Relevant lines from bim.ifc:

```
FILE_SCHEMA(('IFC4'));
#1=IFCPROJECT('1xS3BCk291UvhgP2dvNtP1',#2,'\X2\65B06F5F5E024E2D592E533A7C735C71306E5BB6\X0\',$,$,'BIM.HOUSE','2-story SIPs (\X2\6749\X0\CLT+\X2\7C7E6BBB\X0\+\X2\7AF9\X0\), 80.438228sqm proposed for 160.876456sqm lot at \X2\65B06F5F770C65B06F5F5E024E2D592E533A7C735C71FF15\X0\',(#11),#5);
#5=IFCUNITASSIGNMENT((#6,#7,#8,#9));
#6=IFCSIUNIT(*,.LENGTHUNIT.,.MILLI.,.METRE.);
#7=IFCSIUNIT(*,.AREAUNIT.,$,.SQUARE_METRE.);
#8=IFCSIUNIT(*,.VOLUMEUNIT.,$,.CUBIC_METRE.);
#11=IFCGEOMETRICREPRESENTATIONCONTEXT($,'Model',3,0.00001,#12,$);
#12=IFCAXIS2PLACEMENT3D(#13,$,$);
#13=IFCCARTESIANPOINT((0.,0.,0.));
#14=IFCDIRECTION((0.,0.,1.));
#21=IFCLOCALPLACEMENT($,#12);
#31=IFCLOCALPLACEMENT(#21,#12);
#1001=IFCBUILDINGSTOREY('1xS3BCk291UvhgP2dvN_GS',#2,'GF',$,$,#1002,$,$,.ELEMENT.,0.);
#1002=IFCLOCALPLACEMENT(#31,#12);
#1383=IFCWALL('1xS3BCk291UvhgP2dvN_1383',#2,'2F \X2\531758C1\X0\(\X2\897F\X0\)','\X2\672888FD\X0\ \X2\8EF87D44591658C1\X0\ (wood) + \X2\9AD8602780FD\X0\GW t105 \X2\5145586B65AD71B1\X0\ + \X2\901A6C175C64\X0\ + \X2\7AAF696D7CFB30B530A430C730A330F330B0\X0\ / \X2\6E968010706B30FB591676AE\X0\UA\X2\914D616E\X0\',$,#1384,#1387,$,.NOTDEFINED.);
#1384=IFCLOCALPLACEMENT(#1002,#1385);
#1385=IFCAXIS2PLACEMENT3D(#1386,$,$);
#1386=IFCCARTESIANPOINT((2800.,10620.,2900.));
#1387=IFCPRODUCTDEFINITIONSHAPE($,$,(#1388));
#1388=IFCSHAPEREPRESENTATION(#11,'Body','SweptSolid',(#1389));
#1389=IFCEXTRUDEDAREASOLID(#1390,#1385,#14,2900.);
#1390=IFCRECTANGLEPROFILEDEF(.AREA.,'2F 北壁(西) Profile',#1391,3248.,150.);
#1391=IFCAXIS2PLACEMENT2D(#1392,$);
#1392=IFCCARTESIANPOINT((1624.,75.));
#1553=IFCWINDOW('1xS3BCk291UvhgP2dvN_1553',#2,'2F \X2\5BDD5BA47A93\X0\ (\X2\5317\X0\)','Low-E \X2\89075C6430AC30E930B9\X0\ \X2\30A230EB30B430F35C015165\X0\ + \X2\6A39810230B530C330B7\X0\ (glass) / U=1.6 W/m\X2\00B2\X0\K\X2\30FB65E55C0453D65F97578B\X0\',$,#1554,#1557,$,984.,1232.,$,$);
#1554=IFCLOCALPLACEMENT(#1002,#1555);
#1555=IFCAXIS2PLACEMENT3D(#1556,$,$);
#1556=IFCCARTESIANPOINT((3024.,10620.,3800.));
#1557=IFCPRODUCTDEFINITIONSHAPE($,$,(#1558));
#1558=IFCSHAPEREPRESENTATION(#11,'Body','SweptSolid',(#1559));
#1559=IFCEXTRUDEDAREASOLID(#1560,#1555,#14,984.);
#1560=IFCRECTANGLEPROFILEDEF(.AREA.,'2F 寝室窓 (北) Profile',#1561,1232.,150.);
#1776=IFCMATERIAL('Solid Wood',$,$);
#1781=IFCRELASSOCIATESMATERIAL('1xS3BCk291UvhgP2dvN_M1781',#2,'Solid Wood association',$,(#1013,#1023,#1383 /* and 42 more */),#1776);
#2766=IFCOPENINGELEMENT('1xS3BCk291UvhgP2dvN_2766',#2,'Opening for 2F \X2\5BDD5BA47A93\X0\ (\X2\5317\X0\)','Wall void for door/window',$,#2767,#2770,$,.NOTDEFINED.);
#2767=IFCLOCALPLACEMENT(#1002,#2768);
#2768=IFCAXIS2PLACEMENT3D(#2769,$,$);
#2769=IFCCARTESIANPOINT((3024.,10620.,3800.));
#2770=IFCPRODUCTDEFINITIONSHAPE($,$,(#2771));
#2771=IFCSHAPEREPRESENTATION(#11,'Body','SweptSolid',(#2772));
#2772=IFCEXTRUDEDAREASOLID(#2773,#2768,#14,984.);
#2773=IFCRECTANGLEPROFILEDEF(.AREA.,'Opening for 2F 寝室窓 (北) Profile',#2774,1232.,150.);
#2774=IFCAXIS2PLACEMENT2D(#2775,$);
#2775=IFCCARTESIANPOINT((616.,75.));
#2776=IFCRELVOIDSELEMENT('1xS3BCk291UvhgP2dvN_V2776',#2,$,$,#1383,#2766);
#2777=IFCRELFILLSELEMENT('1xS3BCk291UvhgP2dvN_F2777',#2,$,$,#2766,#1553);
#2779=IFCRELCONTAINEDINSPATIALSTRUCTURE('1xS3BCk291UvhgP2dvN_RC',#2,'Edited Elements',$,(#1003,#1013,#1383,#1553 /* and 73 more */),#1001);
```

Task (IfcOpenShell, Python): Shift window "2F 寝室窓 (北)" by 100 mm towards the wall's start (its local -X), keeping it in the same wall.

```python
import ifcopenshell
import ifcopenshell.api.geometry
import ifcopenshell.util.placement
import ifcopenshell.util.unit

model = ifcopenshell.open("bim.ifc")
unit_scale = ifcopenshell.util.unit.calculate_unit_scale(model)

window = model.by_guid("1xS3BCk291UvhgP2dvN_1553")
opening = window.FillsVoids[0].RelatingOpeningElement
wall = opening.VoidsElements[0].RelatingBuildingElement

wall_matrix = ifcopenshell.util.placement.get_local_placement(wall.ObjectPlacement)
shift = wall_matrix[:3, 0] * -0.1 / unit_scale
before = ifcopenshell.util.placement.get_local_placement(window.ObjectPlacement)[:3, 3].copy()

# The window is not placed relative to its opening, so move both.
for product in (opening, window):
    matrix = ifcopenshell.util.placement.get_local_placement(product.ObjectPlacement)
    matrix[:3, 3] += shift
    ifcopenshell.api.geometry.edit_object_placement(model, product=product, matrix=matrix, is_si=False)

after = ifcopenshell.util.placement.get_local_placement(window.ObjectPlacement)[:3, 3]
print("window moved by", (after - before).round(3) + 0.0)

model.write("bim-out.ifc")
```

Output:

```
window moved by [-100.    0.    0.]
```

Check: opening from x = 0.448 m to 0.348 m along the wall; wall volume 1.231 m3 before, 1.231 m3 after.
